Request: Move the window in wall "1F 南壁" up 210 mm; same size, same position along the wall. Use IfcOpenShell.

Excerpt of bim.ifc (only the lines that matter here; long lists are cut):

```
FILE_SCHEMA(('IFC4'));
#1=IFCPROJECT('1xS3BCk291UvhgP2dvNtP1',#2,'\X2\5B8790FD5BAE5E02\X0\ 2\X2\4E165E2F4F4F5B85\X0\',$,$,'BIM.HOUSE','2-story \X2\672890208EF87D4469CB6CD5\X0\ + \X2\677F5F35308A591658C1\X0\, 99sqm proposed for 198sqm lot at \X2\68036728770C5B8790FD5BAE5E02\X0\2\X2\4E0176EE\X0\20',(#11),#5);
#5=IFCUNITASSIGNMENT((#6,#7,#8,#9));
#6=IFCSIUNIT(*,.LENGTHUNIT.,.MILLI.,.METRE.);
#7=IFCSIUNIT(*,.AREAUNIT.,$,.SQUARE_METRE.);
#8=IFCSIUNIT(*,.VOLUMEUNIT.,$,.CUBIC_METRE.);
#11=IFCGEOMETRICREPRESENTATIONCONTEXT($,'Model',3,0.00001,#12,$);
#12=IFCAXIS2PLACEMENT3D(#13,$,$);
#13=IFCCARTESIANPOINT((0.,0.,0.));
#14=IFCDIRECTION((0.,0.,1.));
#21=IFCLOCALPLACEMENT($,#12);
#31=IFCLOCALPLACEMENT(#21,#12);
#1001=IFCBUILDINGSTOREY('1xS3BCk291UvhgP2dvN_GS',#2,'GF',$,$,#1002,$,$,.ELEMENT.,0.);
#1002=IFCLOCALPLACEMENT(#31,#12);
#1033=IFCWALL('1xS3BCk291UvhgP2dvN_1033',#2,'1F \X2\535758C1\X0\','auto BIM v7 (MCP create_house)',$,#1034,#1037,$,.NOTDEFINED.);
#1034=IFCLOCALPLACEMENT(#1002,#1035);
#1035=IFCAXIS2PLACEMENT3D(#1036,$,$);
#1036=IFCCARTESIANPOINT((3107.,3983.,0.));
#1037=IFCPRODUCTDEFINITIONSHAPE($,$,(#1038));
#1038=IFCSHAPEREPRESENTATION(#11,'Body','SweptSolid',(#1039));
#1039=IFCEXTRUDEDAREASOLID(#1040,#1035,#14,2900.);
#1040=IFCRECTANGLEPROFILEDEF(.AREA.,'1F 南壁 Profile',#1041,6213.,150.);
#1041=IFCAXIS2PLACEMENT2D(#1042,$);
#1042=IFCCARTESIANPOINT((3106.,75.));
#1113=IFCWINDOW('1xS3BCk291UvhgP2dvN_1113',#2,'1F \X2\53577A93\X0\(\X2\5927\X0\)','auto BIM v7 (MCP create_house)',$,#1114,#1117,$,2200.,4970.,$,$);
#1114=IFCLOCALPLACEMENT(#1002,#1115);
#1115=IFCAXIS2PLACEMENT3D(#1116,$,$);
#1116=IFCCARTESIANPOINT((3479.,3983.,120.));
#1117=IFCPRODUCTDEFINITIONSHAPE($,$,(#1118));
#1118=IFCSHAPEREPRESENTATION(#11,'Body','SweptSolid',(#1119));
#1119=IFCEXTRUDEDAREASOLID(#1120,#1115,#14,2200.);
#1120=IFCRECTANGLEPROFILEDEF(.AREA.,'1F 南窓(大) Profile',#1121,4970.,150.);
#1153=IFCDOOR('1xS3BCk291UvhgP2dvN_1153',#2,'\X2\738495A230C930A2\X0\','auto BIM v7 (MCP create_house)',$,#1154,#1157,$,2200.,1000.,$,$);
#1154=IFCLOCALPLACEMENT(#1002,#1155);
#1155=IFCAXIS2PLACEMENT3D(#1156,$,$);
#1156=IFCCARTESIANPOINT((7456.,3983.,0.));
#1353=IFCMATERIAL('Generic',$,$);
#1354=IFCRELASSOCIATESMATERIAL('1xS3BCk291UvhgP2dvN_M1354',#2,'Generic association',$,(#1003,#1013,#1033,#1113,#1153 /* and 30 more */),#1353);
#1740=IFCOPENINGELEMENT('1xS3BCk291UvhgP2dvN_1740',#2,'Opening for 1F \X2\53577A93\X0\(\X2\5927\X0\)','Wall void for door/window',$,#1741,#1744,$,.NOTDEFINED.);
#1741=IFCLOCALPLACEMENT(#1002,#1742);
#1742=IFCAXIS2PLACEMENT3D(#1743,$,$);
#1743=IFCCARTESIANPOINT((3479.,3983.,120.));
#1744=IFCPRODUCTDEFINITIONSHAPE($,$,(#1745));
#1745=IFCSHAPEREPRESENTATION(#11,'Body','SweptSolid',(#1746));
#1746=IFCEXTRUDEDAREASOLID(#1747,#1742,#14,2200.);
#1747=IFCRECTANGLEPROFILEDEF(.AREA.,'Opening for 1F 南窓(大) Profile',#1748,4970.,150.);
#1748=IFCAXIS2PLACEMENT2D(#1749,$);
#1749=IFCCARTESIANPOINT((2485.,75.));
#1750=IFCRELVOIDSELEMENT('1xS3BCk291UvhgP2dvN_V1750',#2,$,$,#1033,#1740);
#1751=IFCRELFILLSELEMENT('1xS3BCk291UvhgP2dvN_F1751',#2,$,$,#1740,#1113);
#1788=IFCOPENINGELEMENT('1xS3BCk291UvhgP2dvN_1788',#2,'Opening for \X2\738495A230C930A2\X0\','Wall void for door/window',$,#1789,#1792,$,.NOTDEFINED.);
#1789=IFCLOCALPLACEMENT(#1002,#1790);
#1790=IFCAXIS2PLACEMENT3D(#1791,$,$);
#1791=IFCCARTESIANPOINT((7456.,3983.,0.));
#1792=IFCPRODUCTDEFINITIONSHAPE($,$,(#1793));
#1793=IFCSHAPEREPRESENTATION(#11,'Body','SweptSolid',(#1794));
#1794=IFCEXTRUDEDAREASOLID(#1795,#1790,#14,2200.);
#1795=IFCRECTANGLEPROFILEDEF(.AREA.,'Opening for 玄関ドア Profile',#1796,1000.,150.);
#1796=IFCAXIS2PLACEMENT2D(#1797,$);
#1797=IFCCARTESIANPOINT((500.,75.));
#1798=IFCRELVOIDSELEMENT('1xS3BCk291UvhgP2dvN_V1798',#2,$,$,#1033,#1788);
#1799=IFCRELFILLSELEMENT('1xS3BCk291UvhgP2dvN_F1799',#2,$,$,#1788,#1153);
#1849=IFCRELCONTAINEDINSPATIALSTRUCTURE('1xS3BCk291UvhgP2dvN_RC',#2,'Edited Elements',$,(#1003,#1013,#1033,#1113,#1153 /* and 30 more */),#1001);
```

```python
import numpy as np
import ifcopenshell
import ifcopenshell.api.geometry
import ifcopenshell.util.placement
import ifcopenshell.util.unit

model = ifcopenshell.open("bim.ifc")
unit_scale = ifcopenshell.util.unit.calculate_unit_scale(model)

window = model.by_guid("1xS3BCk291UvhgP2dvN_1113")
opening = window.FillsVoids[0].RelatingOpeningElement
dz = 0.21 / unit_scale

shift = np.array([0.0, 0.0, dz])
# The window is not placed relative to its opening, so move both.
for product in (opening, window):
    matrix = ifcopenshell.util.placement.get_local_placement(product.ObjectPlacement)
    matrix[:3, 3] += shift
    ifcopenshell.api.geometry.edit_object_placement(model, product=product, matrix=matrix, is_si=False)

print(f"moved by {dz * unit_scale:+.3f} m")

model.write("bim_rev.ifc")
```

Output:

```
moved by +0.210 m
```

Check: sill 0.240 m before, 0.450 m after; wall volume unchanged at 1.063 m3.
